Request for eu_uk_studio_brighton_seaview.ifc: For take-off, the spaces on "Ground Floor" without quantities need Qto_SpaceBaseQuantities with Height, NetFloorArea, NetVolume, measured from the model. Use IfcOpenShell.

First a look at what the model holds.

```python
import ifcopenshell
import ifcopenshell.util.element
import ifcopenshell.util.unit

model = ifcopenshell.open("eu_uk_studio_brighton_seaview.ifc")
print(model.schema)
for unit_type in ("LENGTHUNIT", "AREAUNIT", "VOLUMEUNIT"):
    print(unit_type, ifcopenshell.util.unit.calculate_unit_scale(model, unit_type))
storey = next(s for s in model.by_type("IfcBuildingStorey") if s.Name == "Ground Floor")
spaces = [e for e in ifcopenshell.util.element.get_decomposition(storey) if e.is_a("IfcSpace")]
for e in sorted(spaces, key=lambda e: e.id()):
    print(e.id(), e.is_a(), e.Name, list(ifcopenshell.util.element.get_psets(e, qtos_only=True)), sep=" | ")
```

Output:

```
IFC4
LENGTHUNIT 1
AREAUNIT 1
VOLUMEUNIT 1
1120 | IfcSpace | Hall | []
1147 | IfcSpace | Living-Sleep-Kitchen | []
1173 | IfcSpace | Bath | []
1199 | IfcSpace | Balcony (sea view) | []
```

```python
import ifcopenshell
import ifcopenshell.api.pset
import ifcopenshell.geom
import ifcopenshell.util.element
import ifcopenshell.util.shape
import ifcopenshell.util.unit

model = ifcopenshell.open("eu_uk_studio_brighton_seaview.ifc")
unit_scale = ifcopenshell.util.unit.calculate_unit_scale(model)
area_scale = ifcopenshell.util.unit.calculate_unit_scale(model, "AREAUNIT")
volume_scale = ifcopenshell.util.unit.calculate_unit_scale(model, "VOLUMEUNIT")
settings = ifcopenshell.geom.settings()

storey = next(s for s in model.by_type("IfcBuildingStorey") if s.Name == "Ground Floor")
spaces = [e for e in ifcopenshell.util.element.get_decomposition(storey) if e.is_a("IfcSpace")]

for e in sorted(spaces, key=lambda e: e.id()):
    if ifcopenshell.util.element.get_psets(e, qtos_only=True, should_inherit=False):
        continue
    # Geometry comes back in metres, in the element's own axes.
    shape = ifcopenshell.geom.create_shape(settings, e)
    values = {
        "Height": ifcopenshell.util.shape.get_z(shape.geometry) / unit_scale,
        "NetFloorArea": ifcopenshell.util.shape.get_footprint_area(shape.geometry) / area_scale,
        "NetVolume": ifcopenshell.util.shape.get_volume(shape.geometry) / volume_scale,
    }
    qto = ifcopenshell.api.pset.add_qto(model, product=e, name="Qto_SpaceBaseQuantities")
    ifcopenshell.api.pset.edit_qto(model, qto=qto, properties=values)
    print(e.id(), {k: round(v, 3) for k, v in values.items()})

model.write("eu_uk_studio_brighton_seaview_updated.ifc")
```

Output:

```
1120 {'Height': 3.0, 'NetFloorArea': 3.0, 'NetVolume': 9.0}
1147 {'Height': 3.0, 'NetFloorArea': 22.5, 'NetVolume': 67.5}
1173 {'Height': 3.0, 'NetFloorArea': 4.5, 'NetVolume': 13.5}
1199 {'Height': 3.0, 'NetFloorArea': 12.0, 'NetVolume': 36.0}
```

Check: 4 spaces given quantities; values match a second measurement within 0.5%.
